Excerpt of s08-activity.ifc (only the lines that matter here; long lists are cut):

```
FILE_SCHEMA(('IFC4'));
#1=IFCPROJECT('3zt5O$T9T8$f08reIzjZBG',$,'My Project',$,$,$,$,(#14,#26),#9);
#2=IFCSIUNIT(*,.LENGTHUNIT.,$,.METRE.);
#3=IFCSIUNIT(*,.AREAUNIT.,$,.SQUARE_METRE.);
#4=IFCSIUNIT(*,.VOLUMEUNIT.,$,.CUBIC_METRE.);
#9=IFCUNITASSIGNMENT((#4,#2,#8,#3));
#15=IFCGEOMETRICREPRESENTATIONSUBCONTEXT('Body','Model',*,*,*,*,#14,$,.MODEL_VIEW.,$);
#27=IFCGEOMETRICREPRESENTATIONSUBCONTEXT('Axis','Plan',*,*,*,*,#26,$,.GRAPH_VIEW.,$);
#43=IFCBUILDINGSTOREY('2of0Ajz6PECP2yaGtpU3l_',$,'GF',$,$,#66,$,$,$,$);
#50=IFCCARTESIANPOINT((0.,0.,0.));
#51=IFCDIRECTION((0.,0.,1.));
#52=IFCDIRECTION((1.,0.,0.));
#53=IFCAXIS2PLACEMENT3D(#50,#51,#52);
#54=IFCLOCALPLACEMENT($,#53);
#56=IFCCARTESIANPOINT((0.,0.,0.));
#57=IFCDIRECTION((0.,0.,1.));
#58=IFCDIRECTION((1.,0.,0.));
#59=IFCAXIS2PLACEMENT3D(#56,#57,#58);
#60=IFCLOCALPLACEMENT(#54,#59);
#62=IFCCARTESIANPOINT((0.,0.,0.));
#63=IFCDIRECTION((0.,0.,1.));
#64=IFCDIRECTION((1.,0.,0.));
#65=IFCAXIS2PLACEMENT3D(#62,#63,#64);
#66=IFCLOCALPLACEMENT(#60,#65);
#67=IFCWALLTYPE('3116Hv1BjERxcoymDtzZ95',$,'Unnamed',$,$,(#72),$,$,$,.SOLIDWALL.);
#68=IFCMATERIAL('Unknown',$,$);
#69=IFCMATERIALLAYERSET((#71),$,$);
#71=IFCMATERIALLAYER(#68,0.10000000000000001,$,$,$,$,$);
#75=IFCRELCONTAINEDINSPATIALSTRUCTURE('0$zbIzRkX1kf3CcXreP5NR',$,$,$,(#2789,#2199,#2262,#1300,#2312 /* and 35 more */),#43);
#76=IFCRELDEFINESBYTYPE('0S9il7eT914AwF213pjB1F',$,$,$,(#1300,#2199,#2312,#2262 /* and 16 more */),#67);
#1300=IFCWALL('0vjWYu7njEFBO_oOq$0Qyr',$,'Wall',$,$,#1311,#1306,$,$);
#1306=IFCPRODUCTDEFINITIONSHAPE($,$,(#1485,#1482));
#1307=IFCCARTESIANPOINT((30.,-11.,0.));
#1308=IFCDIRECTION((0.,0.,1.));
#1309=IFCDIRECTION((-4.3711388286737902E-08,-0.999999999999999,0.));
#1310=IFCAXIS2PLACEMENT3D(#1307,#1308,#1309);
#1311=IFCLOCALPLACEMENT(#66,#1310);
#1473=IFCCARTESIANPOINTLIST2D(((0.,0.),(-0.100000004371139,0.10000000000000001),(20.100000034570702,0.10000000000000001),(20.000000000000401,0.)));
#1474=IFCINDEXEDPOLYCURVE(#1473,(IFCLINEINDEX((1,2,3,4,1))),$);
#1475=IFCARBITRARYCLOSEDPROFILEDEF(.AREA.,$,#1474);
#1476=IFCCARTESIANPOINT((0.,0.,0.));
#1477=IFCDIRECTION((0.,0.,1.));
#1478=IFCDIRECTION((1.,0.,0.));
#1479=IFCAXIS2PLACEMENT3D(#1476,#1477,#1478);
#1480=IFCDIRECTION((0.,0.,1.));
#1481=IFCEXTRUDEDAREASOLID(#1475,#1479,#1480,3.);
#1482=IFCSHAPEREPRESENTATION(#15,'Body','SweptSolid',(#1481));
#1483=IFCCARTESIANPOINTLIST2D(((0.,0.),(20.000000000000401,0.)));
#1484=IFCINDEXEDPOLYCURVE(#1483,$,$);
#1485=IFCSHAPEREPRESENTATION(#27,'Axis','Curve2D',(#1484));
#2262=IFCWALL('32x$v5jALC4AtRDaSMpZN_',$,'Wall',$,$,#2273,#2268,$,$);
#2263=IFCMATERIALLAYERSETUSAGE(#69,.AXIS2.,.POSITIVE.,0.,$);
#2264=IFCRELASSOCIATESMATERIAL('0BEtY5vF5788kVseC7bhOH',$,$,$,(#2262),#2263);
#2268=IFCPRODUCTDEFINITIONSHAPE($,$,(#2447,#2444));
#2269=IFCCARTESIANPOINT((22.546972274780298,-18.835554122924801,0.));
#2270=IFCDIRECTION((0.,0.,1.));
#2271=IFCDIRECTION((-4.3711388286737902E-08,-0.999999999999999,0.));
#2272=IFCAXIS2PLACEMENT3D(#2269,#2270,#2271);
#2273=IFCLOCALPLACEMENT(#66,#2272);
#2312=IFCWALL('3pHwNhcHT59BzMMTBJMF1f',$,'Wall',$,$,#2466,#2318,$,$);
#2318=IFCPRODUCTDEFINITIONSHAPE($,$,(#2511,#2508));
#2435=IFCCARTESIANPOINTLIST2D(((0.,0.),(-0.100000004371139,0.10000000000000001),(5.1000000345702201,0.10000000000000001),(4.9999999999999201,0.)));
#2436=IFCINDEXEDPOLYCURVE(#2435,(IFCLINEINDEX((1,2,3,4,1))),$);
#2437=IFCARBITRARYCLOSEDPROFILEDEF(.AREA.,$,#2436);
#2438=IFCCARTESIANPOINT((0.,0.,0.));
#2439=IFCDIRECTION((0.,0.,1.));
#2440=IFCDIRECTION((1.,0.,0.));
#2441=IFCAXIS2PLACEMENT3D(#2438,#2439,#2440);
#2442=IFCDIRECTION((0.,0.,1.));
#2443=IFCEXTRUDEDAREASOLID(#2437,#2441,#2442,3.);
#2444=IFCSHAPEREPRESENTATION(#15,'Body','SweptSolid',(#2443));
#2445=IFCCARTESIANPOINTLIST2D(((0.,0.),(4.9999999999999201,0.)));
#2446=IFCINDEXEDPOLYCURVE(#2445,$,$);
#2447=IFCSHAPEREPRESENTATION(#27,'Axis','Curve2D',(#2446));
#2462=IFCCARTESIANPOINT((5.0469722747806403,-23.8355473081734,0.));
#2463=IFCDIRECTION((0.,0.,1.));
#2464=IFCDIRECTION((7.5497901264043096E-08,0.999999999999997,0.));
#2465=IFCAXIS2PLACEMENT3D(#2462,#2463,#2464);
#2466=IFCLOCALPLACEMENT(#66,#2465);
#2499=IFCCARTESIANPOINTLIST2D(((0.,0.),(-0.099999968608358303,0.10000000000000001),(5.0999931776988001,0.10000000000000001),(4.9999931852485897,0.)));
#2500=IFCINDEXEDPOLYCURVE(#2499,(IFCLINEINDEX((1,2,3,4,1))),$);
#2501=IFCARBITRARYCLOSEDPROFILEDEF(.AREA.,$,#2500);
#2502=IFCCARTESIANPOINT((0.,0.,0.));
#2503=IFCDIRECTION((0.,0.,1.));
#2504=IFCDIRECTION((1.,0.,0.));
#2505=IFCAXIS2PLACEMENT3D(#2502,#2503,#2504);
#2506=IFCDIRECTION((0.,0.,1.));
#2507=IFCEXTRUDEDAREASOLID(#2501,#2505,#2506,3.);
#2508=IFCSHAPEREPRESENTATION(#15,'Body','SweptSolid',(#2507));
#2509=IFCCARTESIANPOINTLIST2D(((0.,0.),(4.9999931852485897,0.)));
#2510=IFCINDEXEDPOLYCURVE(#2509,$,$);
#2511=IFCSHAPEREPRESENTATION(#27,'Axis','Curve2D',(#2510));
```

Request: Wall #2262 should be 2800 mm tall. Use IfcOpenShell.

```python
import ifcopenshell
import ifcopenshell.geom
import ifcopenshell.util.representation
import ifcopenshell.util.shape

model = ifcopenshell.open("s08-activity.ifc")
settings = ifcopenshell.geom.settings()


def volume(element):
    """Net volume in cubic metres, openings subtracted."""
    shape = ifcopenshell.geom.create_shape(settings, element)
    return ifcopenshell.util.shape.get_volume(shape.geometry)


wall = model.by_id(2262)
before = volume(wall)

body = ifcopenshell.util.representation.get_representation(wall, "Model", "Body")
solid = body.Items[0]
old_height = solid.Depth
solid.Depth = 2.8
after = volume(wall)

print(f"height {old_height:g} -> {solid.Depth:g}, volume {before:.3f} -> {after:.3f} m3")

model.write("s08-activity-out.ifc")
```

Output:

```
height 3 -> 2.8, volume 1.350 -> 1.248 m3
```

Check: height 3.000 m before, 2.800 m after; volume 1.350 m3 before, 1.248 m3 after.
